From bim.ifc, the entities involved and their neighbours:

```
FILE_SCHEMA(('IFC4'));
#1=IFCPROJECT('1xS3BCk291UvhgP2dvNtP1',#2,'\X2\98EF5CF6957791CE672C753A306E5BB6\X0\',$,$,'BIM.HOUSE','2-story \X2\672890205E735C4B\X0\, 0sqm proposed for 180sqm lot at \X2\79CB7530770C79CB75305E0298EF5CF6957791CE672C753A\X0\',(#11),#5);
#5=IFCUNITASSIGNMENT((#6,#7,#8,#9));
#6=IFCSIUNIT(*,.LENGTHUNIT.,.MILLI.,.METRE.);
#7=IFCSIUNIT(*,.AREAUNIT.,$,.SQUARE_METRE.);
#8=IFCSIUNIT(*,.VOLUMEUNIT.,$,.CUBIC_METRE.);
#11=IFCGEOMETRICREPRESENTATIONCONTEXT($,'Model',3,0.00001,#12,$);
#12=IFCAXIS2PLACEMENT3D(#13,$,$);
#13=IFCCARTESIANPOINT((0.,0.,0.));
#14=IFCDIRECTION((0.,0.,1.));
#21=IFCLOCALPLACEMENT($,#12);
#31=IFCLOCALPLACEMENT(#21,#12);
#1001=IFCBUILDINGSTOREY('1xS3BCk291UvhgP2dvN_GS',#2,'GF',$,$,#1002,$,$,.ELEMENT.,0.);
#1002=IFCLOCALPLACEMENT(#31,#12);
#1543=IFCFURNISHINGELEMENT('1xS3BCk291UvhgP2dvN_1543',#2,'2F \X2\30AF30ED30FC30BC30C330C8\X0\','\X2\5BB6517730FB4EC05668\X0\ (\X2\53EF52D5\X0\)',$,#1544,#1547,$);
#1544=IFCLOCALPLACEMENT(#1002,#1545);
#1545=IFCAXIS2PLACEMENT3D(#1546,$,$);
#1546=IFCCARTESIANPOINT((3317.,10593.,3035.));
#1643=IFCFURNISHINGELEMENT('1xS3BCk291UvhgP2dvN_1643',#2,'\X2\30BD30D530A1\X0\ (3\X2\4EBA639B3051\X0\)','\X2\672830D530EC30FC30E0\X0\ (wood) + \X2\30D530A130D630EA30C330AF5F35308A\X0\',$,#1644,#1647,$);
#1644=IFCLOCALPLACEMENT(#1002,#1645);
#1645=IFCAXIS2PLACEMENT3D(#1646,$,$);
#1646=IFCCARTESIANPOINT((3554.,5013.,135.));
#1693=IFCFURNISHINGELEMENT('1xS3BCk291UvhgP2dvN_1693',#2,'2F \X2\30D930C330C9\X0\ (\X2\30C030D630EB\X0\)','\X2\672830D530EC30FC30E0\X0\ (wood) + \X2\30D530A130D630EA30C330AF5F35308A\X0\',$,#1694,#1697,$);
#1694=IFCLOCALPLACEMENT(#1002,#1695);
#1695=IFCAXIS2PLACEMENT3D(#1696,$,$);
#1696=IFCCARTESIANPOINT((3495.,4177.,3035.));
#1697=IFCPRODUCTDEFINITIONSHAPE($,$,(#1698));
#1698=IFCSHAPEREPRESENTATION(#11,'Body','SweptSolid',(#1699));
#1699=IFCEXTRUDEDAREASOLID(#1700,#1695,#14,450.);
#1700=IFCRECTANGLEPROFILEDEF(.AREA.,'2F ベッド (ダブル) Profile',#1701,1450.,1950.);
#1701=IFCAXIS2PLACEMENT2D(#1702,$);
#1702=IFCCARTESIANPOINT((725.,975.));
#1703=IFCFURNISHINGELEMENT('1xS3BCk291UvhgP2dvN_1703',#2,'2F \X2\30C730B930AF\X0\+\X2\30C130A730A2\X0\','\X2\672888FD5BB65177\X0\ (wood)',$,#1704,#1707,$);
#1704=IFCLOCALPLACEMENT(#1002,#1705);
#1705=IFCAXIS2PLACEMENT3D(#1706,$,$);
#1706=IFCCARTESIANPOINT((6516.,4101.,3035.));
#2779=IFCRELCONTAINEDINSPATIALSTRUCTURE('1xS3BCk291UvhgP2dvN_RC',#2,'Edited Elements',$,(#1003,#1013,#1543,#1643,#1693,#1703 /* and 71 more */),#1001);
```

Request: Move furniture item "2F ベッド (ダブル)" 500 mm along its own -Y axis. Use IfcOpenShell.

```python
import ifcopenshell
import ifcopenshell.api.geometry
import ifcopenshell.util.placement

model = ifcopenshell.open("bim.ifc")

item = model.by_guid("1xS3BCk291UvhgP2dvN_1693")
matrix = ifcopenshell.util.placement.get_local_placement(item.ObjectPlacement)
matrix[:3, 3] -= matrix[:3, 1] * 500.0
ifcopenshell.api.geometry.edit_object_placement(model, product=item, matrix=matrix, is_si=False)

print(ifcopenshell.util.placement.get_local_placement(item.ObjectPlacement).round(3) + 0.0)

model.write("bim_updated.ifc")
```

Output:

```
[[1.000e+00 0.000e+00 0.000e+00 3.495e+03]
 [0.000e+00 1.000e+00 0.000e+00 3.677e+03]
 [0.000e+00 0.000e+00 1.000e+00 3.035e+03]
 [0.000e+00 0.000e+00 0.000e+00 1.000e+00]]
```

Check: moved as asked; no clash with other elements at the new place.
